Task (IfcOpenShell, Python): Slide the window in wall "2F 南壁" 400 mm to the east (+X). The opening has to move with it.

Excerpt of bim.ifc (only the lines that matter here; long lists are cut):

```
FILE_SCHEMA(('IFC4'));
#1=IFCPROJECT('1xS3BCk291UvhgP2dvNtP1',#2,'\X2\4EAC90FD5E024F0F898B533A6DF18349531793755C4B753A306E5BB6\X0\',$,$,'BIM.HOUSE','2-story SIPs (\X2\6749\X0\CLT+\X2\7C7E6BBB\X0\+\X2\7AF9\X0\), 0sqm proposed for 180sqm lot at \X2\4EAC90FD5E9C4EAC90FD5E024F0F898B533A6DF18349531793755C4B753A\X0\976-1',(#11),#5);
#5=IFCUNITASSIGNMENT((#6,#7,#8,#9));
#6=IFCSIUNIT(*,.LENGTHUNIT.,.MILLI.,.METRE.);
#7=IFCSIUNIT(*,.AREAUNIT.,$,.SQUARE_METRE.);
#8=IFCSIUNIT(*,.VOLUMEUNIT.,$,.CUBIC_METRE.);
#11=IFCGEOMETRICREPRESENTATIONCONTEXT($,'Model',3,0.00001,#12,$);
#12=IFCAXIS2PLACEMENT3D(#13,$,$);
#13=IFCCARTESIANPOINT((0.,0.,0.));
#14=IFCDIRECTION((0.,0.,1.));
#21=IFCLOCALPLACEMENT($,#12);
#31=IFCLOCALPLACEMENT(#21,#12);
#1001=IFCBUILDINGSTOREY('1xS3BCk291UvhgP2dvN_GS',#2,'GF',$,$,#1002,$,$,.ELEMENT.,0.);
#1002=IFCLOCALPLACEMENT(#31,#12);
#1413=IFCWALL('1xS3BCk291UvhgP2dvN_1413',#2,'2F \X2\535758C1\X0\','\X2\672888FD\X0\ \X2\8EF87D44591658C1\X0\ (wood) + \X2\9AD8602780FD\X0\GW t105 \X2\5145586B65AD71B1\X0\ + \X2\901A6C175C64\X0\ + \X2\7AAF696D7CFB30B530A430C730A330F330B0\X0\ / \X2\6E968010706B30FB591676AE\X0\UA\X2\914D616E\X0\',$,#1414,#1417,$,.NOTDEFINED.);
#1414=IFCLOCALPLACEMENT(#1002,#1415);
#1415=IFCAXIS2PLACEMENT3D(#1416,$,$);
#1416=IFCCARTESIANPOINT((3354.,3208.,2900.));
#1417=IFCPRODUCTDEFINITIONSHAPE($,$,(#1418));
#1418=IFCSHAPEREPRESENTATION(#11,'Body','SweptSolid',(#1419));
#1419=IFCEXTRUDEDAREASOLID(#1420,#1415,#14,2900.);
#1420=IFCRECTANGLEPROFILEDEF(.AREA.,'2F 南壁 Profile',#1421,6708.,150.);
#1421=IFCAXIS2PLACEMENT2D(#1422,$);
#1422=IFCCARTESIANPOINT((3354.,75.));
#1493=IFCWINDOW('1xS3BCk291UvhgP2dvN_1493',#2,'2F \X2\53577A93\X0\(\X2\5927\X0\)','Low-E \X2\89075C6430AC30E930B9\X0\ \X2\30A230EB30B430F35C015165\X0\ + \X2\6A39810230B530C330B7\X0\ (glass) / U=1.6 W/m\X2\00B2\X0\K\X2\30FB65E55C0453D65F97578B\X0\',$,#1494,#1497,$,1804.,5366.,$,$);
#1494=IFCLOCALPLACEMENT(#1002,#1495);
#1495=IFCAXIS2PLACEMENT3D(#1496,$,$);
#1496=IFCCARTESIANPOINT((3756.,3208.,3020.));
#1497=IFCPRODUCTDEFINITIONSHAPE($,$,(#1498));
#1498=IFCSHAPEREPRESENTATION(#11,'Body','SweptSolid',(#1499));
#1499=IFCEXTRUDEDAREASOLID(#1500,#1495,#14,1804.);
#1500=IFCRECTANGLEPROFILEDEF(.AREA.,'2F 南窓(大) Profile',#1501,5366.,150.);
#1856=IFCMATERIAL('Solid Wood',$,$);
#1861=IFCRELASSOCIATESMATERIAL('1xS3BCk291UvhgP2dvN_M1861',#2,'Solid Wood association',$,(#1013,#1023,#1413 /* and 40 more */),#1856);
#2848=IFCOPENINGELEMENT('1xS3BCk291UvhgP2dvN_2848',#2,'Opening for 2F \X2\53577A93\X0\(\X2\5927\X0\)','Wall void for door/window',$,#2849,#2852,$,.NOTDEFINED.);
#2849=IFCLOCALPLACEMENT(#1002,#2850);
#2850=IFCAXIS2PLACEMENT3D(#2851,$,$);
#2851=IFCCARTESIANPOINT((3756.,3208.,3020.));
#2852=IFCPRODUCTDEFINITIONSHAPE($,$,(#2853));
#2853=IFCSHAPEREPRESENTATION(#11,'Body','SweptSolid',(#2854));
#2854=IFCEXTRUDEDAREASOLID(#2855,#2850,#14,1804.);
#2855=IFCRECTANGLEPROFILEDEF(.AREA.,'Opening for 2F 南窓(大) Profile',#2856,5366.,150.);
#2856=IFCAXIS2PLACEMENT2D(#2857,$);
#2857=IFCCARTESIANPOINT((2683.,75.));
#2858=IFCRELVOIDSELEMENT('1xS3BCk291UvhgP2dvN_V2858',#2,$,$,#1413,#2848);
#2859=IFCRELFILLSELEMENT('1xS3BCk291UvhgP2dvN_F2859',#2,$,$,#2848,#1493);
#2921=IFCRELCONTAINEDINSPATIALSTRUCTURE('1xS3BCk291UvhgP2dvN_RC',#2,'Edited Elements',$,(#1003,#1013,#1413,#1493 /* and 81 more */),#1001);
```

```python
import ifcopenshell
import ifcopenshell.api.geometry
import ifcopenshell.util.placement
import ifcopenshell.util.unit

model = ifcopenshell.open("bim.ifc")
unit_scale = ifcopenshell.util.unit.calculate_unit_scale(model)

window = model.by_guid("1xS3BCk291UvhgP2dvN_1493")
opening = window.FillsVoids[0].RelatingOpeningElement
wall = opening.VoidsElements[0].RelatingBuildingElement

wall_matrix = ifcopenshell.util.placement.get_local_placement(wall.ObjectPlacement)
shift = wall_matrix[:3, 0] * 0.4 / unit_scale
before = ifcopenshell.util.placement.get_local_placement(window.ObjectPlacement)[:3, 3].copy()

# The window is not placed relative to its opening, so move both.
for product in (opening, window):
    matrix = ifcopenshell.util.placement.get_local_placement(product.ObjectPlacement)
    matrix[:3, 3] += shift
    ifcopenshell.api.geometry.edit_object_placement(model, product=product, matrix=matrix, is_si=False)

after = ifcopenshell.util.placement.get_local_placement(window.ObjectPlacement)[:3, 3]
print("window moved by", (after - before).round(3) + 0.0)

model.write("bim_edited.ifc")
```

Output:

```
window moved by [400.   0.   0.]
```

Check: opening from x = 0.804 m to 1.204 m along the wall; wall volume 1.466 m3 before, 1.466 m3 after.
